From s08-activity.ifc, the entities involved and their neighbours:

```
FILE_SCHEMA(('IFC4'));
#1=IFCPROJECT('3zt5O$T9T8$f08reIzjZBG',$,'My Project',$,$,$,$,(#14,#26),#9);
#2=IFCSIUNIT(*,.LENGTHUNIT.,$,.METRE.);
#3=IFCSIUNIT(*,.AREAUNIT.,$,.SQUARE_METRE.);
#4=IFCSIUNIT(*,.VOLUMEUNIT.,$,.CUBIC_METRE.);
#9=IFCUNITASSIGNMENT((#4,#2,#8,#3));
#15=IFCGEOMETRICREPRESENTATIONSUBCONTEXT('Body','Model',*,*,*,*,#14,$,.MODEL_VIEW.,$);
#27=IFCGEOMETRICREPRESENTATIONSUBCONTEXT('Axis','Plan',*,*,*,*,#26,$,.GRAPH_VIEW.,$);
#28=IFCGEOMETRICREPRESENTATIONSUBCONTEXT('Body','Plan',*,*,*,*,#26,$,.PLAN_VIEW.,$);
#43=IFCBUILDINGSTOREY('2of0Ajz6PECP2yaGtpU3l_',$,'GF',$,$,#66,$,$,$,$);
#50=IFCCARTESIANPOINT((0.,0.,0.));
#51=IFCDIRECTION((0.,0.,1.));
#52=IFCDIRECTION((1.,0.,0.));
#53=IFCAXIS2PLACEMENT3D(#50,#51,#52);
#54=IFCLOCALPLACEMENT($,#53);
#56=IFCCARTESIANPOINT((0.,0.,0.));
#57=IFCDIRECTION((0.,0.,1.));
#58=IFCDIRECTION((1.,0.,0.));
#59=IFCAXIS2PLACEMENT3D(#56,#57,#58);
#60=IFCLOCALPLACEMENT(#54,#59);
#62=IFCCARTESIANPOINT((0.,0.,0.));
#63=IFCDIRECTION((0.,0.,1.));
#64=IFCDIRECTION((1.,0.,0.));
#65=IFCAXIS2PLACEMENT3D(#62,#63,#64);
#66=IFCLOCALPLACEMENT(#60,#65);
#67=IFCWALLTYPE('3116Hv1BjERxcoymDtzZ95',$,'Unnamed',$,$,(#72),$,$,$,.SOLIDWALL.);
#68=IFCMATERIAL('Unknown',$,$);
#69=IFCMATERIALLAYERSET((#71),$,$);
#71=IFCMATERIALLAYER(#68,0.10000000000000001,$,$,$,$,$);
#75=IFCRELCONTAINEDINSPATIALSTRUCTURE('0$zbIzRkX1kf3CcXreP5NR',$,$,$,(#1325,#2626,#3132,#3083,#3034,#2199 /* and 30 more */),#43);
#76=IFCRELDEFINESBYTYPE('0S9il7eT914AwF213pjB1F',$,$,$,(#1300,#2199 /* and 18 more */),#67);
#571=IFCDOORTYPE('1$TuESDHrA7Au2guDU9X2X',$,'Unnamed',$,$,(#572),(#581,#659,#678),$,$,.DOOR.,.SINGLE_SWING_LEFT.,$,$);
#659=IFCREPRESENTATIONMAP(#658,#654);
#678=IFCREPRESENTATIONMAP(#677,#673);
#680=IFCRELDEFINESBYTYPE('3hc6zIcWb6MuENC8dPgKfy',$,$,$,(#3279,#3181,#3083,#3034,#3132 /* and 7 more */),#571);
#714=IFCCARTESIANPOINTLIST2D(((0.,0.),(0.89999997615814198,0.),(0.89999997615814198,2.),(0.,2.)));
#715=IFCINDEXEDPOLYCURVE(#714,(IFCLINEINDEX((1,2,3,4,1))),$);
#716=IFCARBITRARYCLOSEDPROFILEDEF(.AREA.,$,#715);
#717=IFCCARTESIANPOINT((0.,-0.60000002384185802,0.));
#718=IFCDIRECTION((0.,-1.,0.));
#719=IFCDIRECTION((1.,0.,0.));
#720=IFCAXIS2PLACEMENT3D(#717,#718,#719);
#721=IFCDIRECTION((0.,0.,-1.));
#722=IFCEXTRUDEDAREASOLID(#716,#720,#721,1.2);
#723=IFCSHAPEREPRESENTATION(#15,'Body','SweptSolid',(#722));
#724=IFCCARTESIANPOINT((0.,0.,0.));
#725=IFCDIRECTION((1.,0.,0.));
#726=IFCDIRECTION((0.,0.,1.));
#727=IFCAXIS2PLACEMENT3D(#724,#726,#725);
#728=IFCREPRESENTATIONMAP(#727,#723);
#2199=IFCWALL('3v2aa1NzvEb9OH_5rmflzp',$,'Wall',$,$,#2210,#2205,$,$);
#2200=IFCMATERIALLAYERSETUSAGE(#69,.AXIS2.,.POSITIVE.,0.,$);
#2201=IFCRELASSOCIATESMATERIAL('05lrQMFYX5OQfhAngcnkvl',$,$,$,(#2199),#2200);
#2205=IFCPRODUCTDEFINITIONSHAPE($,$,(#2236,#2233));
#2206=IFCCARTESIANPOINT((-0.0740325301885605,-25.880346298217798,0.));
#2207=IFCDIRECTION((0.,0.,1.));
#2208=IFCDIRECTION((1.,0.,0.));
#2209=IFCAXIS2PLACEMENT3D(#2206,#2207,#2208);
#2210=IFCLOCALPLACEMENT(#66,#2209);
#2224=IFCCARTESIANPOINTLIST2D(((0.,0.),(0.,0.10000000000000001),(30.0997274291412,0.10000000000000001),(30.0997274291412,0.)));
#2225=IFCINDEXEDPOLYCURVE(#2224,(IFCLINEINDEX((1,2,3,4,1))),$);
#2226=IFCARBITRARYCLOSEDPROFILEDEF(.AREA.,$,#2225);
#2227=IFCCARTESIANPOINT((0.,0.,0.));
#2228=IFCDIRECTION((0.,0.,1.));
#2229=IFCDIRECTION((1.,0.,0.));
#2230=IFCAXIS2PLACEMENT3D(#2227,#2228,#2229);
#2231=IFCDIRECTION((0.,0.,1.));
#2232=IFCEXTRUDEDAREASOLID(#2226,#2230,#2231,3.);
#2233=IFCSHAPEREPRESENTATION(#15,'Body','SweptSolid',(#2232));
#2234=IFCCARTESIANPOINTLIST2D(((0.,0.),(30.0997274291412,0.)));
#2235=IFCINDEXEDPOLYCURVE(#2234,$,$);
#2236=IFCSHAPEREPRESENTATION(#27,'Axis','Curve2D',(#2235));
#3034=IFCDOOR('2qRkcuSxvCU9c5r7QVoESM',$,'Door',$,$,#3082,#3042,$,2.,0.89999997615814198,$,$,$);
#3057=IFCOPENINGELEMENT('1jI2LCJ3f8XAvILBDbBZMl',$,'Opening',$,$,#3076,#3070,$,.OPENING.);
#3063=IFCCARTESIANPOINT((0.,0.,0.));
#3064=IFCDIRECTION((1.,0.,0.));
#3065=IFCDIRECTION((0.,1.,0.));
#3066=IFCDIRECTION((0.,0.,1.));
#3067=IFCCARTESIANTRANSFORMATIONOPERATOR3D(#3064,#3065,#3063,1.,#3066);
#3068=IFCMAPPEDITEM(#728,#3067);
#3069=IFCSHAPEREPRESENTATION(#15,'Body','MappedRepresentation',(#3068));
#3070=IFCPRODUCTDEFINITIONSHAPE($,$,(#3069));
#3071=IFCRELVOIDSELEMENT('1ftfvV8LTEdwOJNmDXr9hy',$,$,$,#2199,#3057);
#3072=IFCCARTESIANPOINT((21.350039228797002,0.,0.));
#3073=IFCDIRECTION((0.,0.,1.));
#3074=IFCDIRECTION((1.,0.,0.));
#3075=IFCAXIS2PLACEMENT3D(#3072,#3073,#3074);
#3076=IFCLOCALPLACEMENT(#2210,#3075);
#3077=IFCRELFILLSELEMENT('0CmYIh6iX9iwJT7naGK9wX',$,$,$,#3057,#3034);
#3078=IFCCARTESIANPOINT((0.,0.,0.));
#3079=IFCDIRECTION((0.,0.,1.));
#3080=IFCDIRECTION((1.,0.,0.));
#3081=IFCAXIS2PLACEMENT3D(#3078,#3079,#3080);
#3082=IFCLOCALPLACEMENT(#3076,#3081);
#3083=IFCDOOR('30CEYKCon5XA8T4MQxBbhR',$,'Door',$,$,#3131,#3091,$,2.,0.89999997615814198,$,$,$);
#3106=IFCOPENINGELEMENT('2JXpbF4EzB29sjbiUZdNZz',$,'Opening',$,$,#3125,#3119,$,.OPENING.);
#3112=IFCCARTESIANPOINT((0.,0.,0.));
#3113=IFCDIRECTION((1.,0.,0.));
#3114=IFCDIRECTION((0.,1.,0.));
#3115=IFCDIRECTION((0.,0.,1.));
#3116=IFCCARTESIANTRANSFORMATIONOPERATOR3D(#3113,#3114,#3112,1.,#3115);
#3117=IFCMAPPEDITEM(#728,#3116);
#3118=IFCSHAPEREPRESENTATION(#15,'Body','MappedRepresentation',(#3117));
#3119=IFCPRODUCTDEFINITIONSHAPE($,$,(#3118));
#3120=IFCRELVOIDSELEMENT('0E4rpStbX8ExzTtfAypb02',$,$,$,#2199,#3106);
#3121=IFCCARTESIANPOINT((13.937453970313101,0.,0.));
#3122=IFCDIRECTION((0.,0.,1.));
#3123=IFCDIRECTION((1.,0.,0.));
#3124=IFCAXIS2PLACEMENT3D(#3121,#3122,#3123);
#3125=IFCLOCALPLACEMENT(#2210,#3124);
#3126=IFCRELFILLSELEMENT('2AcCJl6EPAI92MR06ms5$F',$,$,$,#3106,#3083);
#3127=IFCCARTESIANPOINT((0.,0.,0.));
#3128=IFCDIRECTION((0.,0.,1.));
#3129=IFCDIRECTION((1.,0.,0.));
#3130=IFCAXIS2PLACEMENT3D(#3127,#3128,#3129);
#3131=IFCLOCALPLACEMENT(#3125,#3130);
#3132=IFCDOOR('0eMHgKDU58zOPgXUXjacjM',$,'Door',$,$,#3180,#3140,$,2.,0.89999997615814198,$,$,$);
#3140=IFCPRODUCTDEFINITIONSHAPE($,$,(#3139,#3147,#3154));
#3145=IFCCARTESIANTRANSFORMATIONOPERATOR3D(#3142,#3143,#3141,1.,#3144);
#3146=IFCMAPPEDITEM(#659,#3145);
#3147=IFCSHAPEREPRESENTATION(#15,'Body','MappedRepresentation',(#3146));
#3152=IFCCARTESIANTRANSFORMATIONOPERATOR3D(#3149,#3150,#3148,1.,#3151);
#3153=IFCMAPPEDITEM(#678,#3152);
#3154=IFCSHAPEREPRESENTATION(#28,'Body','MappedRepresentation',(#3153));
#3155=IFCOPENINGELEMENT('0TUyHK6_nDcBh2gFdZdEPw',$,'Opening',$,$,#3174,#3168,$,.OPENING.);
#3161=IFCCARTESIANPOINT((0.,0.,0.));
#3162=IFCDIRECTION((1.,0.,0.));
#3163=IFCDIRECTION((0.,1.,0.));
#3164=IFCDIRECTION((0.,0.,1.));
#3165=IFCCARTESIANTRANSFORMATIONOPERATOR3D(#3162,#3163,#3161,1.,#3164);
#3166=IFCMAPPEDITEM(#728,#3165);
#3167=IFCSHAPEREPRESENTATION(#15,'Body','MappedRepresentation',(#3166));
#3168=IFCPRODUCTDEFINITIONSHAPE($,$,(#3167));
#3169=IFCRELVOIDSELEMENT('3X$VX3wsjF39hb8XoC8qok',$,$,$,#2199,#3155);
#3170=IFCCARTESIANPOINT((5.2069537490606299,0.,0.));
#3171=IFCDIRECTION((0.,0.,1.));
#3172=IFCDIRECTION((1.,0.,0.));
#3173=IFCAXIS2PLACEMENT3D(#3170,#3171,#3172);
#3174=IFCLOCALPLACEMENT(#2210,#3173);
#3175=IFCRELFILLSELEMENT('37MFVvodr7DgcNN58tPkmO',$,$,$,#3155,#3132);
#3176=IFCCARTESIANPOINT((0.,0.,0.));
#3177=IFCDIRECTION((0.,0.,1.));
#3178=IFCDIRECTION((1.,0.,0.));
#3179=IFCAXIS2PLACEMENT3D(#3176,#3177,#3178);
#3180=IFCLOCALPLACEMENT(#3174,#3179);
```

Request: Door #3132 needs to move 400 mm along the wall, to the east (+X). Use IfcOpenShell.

```python
import ifcopenshell
import ifcopenshell.api.geometry
import ifcopenshell.util.placement
import ifcopenshell.util.unit

model = ifcopenshell.open("s08-activity.ifc")
unit_scale = ifcopenshell.util.unit.calculate_unit_scale(model)

door = model.by_guid("0eMHgKDU58zOPgXUXjacjM")
opening = door.FillsVoids[0].RelatingOpeningElement
wall = opening.VoidsElements[0].RelatingBuildingElement

wall_matrix = ifcopenshell.util.placement.get_local_placement(wall.ObjectPlacement)
shift = wall_matrix[:3, 0] * 0.4 / unit_scale
before = ifcopenshell.util.placement.get_local_placement(door.ObjectPlacement)[:3, 3].copy()

# The door is placed relative to its opening, so it follows when the opening moves.
matrix = ifcopenshell.util.placement.get_local_placement(opening.ObjectPlacement)
matrix[:3, 3] += shift
ifcopenshell.api.geometry.edit_object_placement(
    model, product=opening, matrix=matrix, is_si=False, should_transform_children=True
)

after = ifcopenshell.util.placement.get_local_placement(door.ObjectPlacement)[:3, 3]
print("door moved by", (after - before).round(3) + 0.0)

model.write("s08-activity_v2.ifc")
```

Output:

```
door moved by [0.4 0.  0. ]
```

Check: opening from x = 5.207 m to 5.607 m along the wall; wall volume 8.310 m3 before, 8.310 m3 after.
